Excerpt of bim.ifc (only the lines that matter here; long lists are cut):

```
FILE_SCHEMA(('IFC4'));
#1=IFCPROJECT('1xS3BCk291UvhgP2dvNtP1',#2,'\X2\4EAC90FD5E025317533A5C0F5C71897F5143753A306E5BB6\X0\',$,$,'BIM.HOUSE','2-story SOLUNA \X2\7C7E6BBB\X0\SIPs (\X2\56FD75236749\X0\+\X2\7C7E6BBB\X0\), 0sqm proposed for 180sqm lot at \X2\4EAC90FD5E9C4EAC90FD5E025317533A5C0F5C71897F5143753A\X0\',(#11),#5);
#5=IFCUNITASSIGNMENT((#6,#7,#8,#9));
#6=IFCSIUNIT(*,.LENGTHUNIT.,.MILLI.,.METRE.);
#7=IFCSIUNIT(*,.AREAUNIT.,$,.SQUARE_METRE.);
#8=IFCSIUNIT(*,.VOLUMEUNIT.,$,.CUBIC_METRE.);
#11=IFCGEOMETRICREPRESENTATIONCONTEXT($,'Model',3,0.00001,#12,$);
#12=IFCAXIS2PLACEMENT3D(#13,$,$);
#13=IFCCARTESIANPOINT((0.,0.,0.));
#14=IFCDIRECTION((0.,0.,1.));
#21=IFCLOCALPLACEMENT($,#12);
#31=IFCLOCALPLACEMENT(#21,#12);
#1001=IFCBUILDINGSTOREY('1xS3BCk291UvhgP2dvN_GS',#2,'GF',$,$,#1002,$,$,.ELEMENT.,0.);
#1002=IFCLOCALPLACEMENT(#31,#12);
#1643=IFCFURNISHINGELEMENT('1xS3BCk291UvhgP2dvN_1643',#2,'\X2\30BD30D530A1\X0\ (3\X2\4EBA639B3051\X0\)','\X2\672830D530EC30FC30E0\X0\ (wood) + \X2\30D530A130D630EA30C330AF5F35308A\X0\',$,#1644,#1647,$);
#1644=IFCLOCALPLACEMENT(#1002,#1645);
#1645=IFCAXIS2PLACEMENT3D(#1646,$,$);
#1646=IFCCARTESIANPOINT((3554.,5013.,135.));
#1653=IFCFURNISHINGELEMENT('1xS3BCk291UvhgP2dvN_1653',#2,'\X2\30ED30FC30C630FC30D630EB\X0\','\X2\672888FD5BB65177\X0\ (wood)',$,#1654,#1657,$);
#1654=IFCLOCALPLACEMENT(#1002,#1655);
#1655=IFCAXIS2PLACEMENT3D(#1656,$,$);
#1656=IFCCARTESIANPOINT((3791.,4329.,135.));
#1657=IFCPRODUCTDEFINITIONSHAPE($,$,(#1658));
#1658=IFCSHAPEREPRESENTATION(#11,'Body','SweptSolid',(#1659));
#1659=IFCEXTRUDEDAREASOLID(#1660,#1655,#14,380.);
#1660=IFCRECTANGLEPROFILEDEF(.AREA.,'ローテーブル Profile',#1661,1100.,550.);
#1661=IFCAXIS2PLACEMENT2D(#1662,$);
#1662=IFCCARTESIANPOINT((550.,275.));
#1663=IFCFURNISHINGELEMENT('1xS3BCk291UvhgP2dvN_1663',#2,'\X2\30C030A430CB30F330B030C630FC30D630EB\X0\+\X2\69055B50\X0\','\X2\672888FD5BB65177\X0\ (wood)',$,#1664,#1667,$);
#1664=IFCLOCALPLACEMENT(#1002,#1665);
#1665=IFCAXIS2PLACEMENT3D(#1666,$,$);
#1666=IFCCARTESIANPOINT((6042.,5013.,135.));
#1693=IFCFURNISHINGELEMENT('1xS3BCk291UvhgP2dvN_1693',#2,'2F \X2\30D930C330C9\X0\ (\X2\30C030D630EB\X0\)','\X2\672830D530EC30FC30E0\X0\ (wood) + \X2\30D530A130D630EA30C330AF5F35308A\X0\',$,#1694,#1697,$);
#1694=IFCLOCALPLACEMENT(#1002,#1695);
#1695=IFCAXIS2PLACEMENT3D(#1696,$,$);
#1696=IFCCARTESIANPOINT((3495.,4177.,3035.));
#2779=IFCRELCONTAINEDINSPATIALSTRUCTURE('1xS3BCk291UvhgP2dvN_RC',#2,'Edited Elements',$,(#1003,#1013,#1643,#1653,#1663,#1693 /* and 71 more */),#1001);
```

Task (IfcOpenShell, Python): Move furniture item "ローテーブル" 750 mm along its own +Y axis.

```python
import ifcopenshell
import ifcopenshell.api.geometry
import ifcopenshell.util.placement

model = ifcopenshell.open("bim.ifc")

item = model.by_guid("1xS3BCk291UvhgP2dvN_1653")
matrix = ifcopenshell.util.placement.get_local_placement(item.ObjectPlacement)
matrix[:3, 3] += matrix[:3, 1] * 750.0
ifcopenshell.api.geometry.edit_object_placement(model, product=item, matrix=matrix, is_si=False)

print(ifcopenshell.util.placement.get_local_placement(item.ObjectPlacement).round(3) + 0.0)

model.write("bim-out.ifc")
```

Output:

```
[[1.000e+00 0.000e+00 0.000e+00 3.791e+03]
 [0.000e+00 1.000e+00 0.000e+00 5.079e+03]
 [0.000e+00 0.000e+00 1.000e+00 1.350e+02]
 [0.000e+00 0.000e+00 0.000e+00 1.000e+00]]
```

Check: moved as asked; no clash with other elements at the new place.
